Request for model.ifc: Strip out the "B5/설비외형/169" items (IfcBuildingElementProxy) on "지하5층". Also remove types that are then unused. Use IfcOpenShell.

First a look at what the model holds.

```python
import ifcopenshell
import ifcopenshell.util.element

model = ifcopenshell.open("model.ifc")
print(model.schema)
storey = next(s for s in model.by_type("IfcBuildingStorey") if s.Name == "지하5층")
proxies = [e for e in ifcopenshell.util.element.get_decomposition(storey) if e.is_a("IfcBuildingElementProxy")]
seen = {}
for e in proxies:
    element_type = ifcopenshell.util.element.get_type(e)
    name = element_type.Name if element_type not in (None, e) else None
    seen[name] = seen.get(name, 0) + 1
for name, count in sorted(seen.items(), key=str):
    print(count, "x", name)
```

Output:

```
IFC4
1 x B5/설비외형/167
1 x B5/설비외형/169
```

```python
import ifcopenshell
import ifcopenshell.api.root
import ifcopenshell.util.element

model = ifcopenshell.open("model.ifc")

storey = next(s for s in model.by_type("IfcBuildingStorey") if s.Name == "지하5층")
proxies = [e for e in ifcopenshell.util.element.get_decomposition(storey) if e.is_a("IfcBuildingElementProxy")]
targets = [e for e in proxies if (t := ifcopenshell.util.element.get_type(e)) not in (None, e) and t.Name == "B5/설비외형/169"]
types = {ifcopenshell.util.element.get_type(e) for e in targets} - {None, *targets}

for e in targets:
    ifcopenshell.api.root.remove_product(model, product=e)
print(len(targets), "removed")

unused = [t for t in types if not ifcopenshell.util.element.get_types(t)]
for t in unused:
    ifcopenshell.api.root.remove_product(model, product=t)
print(len(unused), "unused types removed")

model.write("model-out.ifc")
```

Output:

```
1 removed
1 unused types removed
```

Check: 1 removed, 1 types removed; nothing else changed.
